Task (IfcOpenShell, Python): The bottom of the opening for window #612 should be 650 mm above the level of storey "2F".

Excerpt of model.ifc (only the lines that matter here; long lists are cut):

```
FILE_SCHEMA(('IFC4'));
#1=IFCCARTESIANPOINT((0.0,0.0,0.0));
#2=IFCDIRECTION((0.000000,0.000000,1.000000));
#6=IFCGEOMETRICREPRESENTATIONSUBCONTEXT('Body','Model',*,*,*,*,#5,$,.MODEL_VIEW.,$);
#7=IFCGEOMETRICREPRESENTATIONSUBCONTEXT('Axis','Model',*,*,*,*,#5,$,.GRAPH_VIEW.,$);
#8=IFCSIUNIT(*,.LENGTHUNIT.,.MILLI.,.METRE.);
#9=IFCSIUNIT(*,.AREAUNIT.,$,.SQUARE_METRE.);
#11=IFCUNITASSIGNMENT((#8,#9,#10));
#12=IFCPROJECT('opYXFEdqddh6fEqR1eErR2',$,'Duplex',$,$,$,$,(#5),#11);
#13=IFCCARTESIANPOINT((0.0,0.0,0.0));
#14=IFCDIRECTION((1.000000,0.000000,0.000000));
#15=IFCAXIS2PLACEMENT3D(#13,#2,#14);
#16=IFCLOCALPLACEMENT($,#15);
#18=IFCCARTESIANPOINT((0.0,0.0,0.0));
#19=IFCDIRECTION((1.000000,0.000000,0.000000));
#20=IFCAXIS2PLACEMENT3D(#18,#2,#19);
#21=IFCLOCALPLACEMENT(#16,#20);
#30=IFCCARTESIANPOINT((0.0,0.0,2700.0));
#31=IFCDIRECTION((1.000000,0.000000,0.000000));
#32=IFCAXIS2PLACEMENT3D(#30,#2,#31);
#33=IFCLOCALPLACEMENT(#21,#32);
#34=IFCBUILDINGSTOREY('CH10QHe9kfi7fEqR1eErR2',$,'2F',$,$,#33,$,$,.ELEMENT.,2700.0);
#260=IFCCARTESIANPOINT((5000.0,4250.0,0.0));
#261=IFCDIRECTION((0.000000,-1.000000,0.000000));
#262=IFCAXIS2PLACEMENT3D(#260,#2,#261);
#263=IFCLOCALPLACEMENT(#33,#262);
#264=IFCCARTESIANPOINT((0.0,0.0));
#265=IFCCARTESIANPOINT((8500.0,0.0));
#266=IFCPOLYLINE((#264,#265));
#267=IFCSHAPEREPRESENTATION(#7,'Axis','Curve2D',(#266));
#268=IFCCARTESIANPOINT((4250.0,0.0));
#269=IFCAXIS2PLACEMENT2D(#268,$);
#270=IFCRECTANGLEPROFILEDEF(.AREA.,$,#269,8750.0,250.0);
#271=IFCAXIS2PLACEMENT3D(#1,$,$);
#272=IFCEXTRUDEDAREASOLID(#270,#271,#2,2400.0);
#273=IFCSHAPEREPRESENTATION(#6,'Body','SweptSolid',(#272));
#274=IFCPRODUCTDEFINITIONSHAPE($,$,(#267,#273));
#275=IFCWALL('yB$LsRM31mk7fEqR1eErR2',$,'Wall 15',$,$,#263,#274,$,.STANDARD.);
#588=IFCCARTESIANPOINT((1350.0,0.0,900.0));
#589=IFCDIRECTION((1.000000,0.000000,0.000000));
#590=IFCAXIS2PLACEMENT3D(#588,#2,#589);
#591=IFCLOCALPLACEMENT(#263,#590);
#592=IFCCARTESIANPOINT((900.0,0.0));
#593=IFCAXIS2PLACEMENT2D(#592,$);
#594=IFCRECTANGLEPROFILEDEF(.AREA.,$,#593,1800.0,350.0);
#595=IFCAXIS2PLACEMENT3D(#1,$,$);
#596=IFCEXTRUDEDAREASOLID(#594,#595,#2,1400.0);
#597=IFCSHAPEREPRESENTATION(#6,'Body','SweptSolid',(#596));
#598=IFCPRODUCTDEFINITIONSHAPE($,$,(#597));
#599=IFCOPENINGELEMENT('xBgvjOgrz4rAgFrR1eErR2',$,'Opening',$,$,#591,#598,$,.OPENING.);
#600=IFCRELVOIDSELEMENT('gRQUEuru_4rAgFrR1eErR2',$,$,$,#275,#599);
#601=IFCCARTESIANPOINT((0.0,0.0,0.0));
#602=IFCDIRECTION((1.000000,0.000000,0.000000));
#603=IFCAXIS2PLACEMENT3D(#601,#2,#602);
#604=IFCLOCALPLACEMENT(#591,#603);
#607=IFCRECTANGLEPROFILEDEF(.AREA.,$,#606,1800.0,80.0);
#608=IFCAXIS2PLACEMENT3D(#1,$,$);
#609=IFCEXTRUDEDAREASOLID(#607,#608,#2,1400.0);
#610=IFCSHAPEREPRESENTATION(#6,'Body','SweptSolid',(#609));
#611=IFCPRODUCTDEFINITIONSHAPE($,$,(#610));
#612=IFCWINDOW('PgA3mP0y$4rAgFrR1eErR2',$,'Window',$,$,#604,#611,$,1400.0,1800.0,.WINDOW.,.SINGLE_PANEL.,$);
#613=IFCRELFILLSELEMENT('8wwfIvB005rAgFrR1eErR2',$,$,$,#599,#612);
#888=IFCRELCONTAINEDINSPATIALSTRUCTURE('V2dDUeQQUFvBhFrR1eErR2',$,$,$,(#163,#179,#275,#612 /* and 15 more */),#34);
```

```python
import numpy as np
import ifcopenshell
import ifcopenshell.api.geometry
import ifcopenshell.geom
import ifcopenshell.util.element
import ifcopenshell.util.placement
import ifcopenshell.util.shape
import ifcopenshell.util.unit

model = ifcopenshell.open("model.ifc")
unit_scale = ifcopenshell.util.unit.calculate_unit_scale(model)

window = model.by_guid("PgA3mP0y$4rAgFrR1eErR2")
opening = window.FillsVoids[0].RelatingOpeningElement
storey = ifcopenshell.util.element.get_container(window, ifc_class="IfcBuildingStorey")
level = ifcopenshell.util.placement.get_local_placement(storey.ObjectPlacement)[2, 3]

# The opening's origin need not be at the sill, so measure its lowest point.
shape = ifcopenshell.geom.create_shape(ifcopenshell.geom.settings(), opening)
bottom = ifcopenshell.util.shape.get_shape_bottom_elevation(shape, shape.geometry) / unit_scale
dz = level + 0.65 / unit_scale - bottom

shift = np.array([0.0, 0.0, dz])
# The window is placed relative to its opening, so it follows when the opening moves.
matrix = ifcopenshell.util.placement.get_local_placement(opening.ObjectPlacement)
matrix[:3, 3] += shift
ifcopenshell.api.geometry.edit_object_placement(
    model, product=opening, matrix=matrix, is_si=False, should_transform_children=True
)

print(f"moved by {dz * unit_scale:+.3f} m")

model.write("model_updated.ifc")
```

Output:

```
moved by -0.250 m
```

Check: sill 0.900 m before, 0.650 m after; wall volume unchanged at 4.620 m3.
